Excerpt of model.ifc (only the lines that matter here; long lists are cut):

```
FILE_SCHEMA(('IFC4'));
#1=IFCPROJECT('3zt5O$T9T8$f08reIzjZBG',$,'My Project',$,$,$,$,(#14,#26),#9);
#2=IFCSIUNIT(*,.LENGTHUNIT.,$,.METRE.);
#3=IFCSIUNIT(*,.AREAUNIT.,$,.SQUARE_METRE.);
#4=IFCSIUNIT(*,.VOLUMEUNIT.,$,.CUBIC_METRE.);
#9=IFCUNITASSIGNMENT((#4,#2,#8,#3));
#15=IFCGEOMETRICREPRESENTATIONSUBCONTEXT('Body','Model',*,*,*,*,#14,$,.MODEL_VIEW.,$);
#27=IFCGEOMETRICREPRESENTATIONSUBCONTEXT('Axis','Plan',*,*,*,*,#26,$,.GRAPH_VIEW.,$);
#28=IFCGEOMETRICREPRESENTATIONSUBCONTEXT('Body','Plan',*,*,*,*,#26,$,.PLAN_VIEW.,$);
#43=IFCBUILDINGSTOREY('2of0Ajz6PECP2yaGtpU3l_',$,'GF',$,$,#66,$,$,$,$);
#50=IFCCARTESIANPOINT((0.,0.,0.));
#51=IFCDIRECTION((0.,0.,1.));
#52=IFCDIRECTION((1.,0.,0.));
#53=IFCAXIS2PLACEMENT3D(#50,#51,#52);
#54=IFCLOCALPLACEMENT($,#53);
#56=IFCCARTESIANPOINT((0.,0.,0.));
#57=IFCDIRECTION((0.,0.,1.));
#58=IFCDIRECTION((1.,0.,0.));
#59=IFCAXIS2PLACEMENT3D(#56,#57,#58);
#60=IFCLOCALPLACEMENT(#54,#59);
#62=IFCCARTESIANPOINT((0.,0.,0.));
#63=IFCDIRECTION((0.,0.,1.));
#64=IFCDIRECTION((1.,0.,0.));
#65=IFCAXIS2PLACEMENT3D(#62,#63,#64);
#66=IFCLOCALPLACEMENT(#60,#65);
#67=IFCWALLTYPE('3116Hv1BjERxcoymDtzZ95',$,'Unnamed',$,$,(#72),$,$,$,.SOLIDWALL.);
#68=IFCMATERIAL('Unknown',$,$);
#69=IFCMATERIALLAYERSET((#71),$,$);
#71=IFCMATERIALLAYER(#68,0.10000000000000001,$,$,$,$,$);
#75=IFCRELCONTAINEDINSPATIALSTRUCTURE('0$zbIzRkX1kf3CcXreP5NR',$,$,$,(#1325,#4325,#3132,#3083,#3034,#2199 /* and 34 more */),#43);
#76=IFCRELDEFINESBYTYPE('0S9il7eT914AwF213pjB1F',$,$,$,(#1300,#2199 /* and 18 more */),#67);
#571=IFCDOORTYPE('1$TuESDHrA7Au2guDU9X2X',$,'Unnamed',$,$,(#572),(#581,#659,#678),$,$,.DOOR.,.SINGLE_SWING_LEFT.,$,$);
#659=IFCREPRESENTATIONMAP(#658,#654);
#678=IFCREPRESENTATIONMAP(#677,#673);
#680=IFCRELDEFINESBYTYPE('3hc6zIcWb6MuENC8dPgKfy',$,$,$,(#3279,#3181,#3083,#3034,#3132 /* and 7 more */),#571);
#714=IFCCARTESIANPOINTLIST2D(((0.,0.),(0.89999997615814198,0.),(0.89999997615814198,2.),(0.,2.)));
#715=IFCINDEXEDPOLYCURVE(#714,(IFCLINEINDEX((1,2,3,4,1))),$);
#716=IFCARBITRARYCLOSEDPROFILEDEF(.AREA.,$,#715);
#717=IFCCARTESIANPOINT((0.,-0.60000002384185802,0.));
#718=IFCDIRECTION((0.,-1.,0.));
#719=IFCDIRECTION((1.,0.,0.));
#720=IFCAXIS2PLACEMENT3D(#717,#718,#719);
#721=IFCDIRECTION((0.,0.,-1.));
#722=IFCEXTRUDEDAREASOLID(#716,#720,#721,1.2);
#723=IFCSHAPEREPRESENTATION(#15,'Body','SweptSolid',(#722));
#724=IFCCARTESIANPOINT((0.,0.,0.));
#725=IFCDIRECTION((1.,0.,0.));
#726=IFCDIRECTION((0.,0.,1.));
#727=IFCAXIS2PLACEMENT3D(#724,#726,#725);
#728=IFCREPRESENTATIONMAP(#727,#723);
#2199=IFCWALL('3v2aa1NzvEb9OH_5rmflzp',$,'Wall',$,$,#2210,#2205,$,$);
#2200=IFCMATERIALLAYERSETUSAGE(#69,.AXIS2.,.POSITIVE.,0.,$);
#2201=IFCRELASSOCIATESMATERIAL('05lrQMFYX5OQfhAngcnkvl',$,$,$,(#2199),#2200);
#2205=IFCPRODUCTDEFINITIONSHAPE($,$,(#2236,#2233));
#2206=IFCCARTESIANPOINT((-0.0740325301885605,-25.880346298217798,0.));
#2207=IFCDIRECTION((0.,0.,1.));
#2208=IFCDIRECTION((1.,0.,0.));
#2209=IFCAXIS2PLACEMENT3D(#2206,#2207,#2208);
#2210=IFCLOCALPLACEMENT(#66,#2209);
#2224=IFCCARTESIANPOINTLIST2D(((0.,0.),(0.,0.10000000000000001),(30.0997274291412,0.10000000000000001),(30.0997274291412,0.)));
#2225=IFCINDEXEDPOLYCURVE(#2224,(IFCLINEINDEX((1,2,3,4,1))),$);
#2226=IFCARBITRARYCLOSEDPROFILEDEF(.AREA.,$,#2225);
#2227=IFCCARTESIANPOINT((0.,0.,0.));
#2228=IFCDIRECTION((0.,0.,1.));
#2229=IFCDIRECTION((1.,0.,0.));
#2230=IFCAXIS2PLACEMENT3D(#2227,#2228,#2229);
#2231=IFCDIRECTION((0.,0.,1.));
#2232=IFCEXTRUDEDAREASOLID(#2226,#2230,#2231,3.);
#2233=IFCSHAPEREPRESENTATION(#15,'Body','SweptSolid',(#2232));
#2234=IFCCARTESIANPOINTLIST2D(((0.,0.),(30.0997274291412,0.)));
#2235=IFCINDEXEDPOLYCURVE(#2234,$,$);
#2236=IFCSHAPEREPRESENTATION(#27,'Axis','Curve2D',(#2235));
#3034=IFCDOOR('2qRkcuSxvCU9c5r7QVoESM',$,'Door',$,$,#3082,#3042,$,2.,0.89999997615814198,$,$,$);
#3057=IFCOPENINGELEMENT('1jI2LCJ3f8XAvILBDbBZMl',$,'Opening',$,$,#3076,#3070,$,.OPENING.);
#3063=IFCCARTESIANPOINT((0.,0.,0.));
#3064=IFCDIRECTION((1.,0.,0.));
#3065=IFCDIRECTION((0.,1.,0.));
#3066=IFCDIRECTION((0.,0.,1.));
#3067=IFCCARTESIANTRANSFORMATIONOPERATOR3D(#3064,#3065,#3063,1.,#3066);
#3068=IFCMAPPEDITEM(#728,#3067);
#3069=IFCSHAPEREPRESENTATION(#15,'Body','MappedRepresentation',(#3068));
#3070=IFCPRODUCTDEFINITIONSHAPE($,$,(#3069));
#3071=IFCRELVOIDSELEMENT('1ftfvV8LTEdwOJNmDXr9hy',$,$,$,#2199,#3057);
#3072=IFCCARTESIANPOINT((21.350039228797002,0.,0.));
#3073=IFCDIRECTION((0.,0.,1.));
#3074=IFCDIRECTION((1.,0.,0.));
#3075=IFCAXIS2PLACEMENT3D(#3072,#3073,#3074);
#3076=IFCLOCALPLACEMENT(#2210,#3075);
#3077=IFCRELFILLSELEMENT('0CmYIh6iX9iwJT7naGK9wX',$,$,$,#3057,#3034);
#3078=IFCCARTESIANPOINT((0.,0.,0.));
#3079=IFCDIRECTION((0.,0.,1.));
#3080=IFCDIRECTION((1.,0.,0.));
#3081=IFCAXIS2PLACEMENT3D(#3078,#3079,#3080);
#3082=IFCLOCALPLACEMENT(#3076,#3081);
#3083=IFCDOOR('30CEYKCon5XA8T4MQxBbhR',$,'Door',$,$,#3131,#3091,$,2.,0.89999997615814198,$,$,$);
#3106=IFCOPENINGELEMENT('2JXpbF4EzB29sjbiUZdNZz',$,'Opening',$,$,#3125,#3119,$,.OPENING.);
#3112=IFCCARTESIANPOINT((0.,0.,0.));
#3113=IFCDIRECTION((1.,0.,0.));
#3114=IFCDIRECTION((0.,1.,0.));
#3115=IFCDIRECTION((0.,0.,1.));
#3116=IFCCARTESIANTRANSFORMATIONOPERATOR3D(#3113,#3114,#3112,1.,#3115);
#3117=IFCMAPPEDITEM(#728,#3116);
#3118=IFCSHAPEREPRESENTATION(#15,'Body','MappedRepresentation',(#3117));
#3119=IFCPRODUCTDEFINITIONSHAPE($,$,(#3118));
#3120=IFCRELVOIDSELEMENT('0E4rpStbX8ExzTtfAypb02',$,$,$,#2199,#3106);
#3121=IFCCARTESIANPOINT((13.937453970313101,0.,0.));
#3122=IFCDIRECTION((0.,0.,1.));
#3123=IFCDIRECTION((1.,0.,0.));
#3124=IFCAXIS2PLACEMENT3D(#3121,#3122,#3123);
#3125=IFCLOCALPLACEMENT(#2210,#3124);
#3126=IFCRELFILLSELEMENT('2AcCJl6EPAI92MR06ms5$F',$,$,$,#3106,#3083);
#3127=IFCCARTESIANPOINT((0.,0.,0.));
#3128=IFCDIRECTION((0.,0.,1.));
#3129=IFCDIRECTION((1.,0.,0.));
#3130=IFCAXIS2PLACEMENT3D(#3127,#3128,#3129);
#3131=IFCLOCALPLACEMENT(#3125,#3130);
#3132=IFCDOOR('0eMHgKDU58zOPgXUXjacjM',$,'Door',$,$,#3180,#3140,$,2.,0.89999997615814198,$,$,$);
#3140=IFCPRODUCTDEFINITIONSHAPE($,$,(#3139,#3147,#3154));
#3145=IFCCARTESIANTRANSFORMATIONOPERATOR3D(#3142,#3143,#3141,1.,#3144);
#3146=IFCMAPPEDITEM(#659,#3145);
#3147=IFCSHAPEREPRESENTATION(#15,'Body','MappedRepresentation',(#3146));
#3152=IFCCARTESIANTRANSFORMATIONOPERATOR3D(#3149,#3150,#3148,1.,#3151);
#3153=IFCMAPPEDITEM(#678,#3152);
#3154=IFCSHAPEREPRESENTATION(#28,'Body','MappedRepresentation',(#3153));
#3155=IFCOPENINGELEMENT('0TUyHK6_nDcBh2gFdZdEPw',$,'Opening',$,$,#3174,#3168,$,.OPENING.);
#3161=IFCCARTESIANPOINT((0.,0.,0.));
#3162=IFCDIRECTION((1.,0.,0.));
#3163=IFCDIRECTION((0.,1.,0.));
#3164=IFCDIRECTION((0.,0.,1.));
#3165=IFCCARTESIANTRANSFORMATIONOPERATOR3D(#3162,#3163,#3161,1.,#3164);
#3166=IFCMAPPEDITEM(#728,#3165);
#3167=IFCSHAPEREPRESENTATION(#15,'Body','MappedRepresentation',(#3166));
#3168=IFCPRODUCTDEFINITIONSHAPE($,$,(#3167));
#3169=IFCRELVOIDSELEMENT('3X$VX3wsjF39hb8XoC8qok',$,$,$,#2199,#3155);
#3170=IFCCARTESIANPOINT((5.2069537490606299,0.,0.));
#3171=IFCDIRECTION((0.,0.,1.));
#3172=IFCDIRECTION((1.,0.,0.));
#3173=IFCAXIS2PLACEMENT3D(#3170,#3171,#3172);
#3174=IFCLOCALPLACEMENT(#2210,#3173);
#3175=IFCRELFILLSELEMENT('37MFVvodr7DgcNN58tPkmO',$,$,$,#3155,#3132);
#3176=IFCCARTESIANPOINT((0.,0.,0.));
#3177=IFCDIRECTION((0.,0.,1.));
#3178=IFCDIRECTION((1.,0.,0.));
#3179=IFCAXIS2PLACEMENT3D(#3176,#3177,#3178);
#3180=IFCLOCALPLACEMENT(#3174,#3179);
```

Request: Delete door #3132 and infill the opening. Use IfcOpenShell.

```python
import ifcopenshell
import ifcopenshell.api.feature
import ifcopenshell.api.root
import ifcopenshell.geom
import ifcopenshell.util.shape

model = ifcopenshell.open("model.ifc")
settings = ifcopenshell.geom.settings()


def volume(element):
    """Net volume in cubic metres, openings subtracted."""
    shape = ifcopenshell.geom.create_shape(settings, element)
    return ifcopenshell.util.shape.get_volume(shape.geometry)


door = model.by_guid("0eMHgKDU58zOPgXUXjacjM")
opening = door.FillsVoids[0].RelatingOpeningElement
wall = opening.VoidsElements[0].RelatingBuildingElement
before = volume(wall)

ifcopenshell.api.root.remove_product(model, product=door)
ifcopenshell.api.feature.remove_feature(model, feature=opening)

after = volume(wall)

print(f"wall volume {before:.3f} -> {after:.3f} m3")

model.write("model-out.ifc")
```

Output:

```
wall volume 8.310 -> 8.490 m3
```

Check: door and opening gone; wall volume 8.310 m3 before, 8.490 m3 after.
